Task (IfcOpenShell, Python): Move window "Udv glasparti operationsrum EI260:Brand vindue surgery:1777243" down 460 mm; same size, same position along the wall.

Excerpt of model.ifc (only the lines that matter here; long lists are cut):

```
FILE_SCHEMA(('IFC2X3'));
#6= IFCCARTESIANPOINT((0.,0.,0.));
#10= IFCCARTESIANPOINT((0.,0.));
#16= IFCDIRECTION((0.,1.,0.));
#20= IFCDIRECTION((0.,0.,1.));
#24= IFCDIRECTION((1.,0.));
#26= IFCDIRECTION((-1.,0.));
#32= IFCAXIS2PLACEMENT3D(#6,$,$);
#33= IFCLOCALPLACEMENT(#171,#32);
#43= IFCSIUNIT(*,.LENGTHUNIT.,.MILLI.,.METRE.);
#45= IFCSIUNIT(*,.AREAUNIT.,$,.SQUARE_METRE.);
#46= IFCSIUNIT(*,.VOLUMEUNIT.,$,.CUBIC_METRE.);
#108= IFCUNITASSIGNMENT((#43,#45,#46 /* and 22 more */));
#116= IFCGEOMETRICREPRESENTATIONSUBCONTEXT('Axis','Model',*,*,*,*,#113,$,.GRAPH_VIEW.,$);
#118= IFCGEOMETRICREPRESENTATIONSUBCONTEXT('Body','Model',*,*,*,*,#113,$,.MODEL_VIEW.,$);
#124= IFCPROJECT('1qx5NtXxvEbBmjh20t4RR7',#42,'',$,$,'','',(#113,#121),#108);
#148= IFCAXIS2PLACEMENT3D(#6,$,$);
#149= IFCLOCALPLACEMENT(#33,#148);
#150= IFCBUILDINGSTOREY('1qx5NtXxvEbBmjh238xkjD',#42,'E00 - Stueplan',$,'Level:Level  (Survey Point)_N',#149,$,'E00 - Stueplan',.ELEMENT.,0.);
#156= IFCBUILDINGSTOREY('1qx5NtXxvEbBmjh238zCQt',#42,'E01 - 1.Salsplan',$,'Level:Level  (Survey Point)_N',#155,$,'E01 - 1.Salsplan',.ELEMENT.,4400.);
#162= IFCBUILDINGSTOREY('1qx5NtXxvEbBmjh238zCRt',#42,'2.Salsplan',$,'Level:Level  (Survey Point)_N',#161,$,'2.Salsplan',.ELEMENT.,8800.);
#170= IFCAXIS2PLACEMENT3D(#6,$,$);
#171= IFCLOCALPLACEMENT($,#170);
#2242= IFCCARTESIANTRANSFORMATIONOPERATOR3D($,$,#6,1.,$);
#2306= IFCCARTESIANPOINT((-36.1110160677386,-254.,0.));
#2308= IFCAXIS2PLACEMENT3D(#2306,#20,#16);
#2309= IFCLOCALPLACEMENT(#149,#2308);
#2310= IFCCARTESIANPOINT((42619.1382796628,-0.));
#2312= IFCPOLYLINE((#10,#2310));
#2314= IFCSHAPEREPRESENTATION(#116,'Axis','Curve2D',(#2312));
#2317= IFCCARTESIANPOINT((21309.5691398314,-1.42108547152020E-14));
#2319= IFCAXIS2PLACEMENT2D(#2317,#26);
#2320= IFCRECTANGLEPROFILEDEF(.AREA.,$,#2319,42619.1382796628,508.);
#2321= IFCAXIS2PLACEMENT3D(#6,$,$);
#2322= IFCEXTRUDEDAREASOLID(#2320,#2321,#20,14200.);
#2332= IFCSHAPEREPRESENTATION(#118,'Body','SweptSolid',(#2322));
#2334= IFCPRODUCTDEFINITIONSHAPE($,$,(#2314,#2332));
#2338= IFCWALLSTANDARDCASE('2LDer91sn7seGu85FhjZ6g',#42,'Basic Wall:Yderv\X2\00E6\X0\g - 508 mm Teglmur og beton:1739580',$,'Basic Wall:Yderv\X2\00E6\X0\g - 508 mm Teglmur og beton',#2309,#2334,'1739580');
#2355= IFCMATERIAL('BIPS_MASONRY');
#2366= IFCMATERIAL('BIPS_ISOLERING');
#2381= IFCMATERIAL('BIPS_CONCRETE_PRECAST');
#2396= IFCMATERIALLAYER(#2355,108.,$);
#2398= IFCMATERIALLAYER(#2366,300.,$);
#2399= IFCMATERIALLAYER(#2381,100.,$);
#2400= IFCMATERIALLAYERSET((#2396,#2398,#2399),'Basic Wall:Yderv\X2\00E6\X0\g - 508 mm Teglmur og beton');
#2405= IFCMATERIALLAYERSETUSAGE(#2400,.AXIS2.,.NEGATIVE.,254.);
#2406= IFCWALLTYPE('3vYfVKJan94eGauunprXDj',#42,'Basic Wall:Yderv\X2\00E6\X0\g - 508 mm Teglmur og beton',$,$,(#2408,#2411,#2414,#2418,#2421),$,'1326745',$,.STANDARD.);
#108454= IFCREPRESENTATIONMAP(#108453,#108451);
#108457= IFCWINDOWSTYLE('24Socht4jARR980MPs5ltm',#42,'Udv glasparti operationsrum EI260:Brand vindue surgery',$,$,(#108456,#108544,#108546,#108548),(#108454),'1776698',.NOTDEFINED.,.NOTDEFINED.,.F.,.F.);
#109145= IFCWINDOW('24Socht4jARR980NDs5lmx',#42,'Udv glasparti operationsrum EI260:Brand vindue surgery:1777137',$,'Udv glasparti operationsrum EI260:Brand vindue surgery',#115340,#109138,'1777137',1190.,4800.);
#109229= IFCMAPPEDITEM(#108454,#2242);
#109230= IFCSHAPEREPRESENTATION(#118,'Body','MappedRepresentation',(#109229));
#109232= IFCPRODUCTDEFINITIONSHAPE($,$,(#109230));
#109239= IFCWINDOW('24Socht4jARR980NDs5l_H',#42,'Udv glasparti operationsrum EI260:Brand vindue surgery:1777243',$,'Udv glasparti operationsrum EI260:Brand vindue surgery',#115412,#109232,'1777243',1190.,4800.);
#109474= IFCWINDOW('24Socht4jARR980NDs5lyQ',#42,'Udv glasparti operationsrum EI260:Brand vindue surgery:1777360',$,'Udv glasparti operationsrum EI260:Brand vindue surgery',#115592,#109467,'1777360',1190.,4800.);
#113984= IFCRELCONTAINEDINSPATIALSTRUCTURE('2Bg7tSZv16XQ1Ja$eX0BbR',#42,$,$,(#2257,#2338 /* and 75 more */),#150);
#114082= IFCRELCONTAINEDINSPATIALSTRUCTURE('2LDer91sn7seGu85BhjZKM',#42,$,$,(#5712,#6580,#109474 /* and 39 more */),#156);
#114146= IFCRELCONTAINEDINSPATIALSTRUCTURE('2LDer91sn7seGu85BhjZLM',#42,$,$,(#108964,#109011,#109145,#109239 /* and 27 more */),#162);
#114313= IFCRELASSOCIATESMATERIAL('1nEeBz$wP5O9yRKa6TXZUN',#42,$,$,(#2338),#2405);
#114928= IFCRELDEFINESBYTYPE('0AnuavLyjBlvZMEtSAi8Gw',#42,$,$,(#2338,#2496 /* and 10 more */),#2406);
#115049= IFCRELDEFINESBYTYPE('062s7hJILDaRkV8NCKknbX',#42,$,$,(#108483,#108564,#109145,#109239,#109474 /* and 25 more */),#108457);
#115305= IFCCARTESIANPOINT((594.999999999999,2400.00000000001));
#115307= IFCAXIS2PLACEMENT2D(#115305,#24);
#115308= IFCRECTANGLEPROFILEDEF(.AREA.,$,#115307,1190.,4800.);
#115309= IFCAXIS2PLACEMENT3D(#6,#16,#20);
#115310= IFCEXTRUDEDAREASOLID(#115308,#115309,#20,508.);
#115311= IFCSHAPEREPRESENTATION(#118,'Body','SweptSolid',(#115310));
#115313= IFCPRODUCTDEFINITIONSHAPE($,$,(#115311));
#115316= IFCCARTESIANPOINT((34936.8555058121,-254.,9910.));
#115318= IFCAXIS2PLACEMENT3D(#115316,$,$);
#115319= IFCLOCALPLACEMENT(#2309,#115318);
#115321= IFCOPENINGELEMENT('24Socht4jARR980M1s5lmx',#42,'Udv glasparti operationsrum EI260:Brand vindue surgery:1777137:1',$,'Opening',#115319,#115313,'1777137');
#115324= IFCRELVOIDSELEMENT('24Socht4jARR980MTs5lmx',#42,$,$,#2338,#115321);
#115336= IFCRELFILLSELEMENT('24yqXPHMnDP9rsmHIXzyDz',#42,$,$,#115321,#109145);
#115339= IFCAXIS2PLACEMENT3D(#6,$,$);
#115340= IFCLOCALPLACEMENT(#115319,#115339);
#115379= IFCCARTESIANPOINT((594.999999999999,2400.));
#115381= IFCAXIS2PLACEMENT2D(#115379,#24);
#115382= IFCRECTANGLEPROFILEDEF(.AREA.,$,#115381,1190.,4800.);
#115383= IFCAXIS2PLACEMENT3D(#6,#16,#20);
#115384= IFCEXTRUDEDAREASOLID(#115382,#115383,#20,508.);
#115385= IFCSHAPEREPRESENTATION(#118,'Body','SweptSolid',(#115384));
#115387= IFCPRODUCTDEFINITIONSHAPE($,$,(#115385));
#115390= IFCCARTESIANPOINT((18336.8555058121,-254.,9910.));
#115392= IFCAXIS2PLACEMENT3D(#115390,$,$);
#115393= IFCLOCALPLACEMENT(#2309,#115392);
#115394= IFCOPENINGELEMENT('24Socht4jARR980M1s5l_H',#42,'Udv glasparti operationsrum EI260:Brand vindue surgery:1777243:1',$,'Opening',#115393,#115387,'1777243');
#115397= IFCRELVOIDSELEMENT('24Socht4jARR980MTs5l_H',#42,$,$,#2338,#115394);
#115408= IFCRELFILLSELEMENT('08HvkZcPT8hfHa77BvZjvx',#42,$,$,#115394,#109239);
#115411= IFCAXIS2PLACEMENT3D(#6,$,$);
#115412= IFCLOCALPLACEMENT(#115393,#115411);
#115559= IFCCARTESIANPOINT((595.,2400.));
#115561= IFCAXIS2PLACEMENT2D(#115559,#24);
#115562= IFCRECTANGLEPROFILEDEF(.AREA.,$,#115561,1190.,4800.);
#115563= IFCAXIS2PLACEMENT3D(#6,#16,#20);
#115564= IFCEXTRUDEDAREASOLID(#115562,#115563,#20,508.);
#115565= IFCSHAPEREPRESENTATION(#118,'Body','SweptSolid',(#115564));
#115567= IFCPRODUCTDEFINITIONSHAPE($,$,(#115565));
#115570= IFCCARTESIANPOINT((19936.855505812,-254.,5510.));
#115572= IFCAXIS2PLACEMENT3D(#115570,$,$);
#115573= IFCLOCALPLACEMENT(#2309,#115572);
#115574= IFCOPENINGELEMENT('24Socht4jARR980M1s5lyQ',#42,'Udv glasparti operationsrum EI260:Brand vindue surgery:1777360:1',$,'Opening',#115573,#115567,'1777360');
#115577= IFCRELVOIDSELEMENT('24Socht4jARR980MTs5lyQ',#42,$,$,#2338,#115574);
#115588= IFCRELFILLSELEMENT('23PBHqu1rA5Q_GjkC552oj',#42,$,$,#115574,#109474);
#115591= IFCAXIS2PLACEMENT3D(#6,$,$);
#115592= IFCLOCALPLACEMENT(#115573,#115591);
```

```python
import numpy as np
import ifcopenshell
import ifcopenshell.api.geometry
import ifcopenshell.util.placement
import ifcopenshell.util.unit

model = ifcopenshell.open("model.ifc")
unit_scale = ifcopenshell.util.unit.calculate_unit_scale(model)

window = model.by_id(109239)
opening = window.FillsVoids[0].RelatingOpeningElement
dz = -0.46 / unit_scale

shift = np.array([0.0, 0.0, dz])
# The window is placed relative to its opening, so it follows when the opening moves.
matrix = ifcopenshell.util.placement.get_local_placement(opening.ObjectPlacement)
matrix[:3, 3] += shift
ifcopenshell.api.geometry.edit_object_placement(
    model, product=opening, matrix=matrix, is_si=False, should_transform_children=True
)

print(f"moved by {dz * unit_scale:+.3f} m")

model.write("model-out.ifc")
```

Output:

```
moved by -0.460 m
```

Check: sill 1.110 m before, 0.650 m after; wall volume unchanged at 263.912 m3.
